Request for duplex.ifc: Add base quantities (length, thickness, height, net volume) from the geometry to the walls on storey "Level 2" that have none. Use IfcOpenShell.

First a look at what the model holds.

```python
import ifcopenshell
import ifcopenshell.util.element
import ifcopenshell.util.unit

model = ifcopenshell.open("duplex.ifc")
print(model.schema)
for unit_type in ("LENGTHUNIT", "AREAUNIT", "VOLUMEUNIT"):
    print(unit_type, ifcopenshell.util.unit.calculate_unit_scale(model, unit_type))
storey = next(s for s in model.by_type("IfcBuildingStorey") if s.Name == "Level 2")
walls = [e for e in ifcopenshell.util.element.get_decomposition(storey) if e.is_a("IfcWall")]
for e in sorted(walls, key=lambda e: e.id()):
    print(e.id(), e.is_a(), e.Name, list(ifcopenshell.util.element.get_psets(e, qtos_only=True)), sep=" | ")
```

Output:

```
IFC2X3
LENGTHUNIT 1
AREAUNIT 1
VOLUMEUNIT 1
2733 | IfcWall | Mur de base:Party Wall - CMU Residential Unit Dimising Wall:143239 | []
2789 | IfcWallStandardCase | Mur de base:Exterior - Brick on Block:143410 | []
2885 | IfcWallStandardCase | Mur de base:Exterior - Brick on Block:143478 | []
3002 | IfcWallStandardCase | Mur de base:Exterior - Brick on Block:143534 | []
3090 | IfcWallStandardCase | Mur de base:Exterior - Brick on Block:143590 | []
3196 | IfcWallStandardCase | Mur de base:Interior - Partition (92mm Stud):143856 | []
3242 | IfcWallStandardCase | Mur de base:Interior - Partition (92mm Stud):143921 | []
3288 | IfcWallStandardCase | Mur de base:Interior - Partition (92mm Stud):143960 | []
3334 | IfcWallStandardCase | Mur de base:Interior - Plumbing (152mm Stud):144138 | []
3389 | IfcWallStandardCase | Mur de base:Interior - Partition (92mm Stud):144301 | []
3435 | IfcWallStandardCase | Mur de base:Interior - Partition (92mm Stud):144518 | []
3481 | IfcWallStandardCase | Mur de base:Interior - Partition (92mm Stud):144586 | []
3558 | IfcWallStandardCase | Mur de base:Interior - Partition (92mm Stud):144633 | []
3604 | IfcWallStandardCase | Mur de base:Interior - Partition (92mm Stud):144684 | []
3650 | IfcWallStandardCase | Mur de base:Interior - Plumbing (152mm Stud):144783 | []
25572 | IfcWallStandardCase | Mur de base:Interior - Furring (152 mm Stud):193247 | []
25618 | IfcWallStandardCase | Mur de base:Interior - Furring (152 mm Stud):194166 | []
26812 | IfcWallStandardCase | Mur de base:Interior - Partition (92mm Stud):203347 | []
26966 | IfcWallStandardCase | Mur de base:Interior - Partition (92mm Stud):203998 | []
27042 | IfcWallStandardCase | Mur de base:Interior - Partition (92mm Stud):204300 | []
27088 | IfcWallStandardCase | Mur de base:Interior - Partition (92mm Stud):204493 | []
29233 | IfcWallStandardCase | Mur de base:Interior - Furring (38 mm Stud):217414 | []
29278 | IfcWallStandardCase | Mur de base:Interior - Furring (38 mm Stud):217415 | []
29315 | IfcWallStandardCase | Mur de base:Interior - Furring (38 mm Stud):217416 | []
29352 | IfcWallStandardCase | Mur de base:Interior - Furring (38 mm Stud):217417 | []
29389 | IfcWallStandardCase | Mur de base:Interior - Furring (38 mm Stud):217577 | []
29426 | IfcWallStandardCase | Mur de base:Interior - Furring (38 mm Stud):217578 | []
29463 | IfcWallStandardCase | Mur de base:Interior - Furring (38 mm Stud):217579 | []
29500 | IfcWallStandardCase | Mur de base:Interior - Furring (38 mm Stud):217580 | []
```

```python
import ifcopenshell
import ifcopenshell.api.pset
import ifcopenshell.geom
import ifcopenshell.util.element
import ifcopenshell.util.shape
import ifcopenshell.util.unit

model = ifcopenshell.open("duplex.ifc")
unit_scale = ifcopenshell.util.unit.calculate_unit_scale(model)
volume_scale = ifcopenshell.util.unit.calculate_unit_scale(model, "VOLUMEUNIT")
settings = ifcopenshell.geom.settings()

storey = next(s for s in model.by_type("IfcBuildingStorey") if s.Name == "Level 2")
walls = [e for e in ifcopenshell.util.element.get_decomposition(storey) if e.is_a("IfcWall")]

for e in sorted(walls, key=lambda e: e.id()):
    if ifcopenshell.util.element.get_psets(e, qtos_only=True, should_inherit=False):
        continue
    # Geometry comes back in metres, in the element's own axes.
    shape = ifcopenshell.geom.create_shape(settings, e)
    values = {
        "Length": ifcopenshell.util.shape.get_x(shape.geometry) / unit_scale,
        "Width": ifcopenshell.util.shape.get_y(shape.geometry) / unit_scale,
        "Height": ifcopenshell.util.shape.get_z(shape.geometry) / unit_scale,
        "NetVolume": ifcopenshell.util.shape.get_volume(shape.geometry) / volume_scale,
    }
    qto = ifcopenshell.api.pset.add_qto(model, product=e, name="BaseQuantities")
    ifcopenshell.api.pset.edit_qto(model, qto=qto, properties=values)
    print(e.id(), {k: round(v, 3) for k, v in values.items()})

model.write("duplex-out.ifc")
```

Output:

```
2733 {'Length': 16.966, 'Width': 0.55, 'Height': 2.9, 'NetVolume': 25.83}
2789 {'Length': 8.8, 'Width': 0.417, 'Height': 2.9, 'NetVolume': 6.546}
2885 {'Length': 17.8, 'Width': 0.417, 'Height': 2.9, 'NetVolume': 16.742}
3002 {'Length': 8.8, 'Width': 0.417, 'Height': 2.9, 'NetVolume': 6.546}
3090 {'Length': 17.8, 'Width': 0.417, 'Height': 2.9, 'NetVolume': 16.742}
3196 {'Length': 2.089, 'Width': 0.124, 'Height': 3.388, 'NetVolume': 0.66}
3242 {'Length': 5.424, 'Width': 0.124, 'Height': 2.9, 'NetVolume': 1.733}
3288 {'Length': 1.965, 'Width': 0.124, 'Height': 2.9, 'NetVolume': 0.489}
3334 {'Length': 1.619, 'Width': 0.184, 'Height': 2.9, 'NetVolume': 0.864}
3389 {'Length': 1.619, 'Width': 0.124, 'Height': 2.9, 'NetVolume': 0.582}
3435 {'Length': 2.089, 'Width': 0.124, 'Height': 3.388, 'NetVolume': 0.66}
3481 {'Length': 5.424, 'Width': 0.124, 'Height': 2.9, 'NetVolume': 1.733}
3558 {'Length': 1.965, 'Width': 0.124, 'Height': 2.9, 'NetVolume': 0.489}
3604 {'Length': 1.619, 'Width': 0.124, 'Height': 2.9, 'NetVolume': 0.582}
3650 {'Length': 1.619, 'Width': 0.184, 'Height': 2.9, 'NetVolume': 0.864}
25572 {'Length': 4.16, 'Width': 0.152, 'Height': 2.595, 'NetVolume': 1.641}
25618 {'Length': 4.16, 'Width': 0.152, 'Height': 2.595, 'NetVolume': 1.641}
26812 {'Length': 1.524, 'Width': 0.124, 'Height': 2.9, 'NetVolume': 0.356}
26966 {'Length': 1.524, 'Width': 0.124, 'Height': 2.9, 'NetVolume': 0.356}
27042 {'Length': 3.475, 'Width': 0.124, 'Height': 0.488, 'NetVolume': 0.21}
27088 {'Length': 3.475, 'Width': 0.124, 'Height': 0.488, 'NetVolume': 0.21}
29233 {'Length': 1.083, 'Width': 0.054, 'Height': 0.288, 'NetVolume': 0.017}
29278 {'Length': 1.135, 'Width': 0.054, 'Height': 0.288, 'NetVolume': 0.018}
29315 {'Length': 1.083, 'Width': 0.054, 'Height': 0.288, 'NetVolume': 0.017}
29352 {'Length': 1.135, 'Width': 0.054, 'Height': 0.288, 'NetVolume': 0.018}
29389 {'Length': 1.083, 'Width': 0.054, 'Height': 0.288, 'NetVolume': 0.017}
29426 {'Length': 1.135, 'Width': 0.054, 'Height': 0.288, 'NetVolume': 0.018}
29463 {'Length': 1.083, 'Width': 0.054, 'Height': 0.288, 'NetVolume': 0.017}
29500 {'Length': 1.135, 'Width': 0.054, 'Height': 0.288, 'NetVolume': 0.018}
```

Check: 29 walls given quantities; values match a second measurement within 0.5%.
